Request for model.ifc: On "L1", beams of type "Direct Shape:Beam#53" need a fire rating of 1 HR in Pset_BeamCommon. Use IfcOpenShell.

First a look at what the model holds.

```python
import ifcopenshell
import ifcopenshell.util.element

model = ifcopenshell.open("model.ifc")
print(model.schema)
storey = next(s for s in model.by_type("IfcBuildingStorey") if s.Name == "L1")
beams = [e for e in ifcopenshell.util.element.get_decomposition(storey) if e.is_a("IfcBeam")]
seen = {}
for e in beams:
    element_type = ifcopenshell.util.element.get_type(e)
    key = (element_type.Name if element_type != e and element_type else None, ifcopenshell.util.element.get_pset(e, "Pset_BeamCommon", "FireRating"))
    seen[key] = seen.get(key, 0) + 1
for (name, value), count in sorted(seen.items(), key=str):
    print(count, "x", name, "|", value)
```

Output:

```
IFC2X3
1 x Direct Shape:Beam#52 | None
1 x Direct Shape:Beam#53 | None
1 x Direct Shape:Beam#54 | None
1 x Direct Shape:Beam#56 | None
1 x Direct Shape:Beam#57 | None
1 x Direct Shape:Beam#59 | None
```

```python
import ifcopenshell
import ifcopenshell.api.pset
import ifcopenshell.util.element

model = ifcopenshell.open("model.ifc")

storey = next(s for s in model.by_type("IfcBuildingStorey") if s.Name == "L1")
beams = [e for e in ifcopenshell.util.element.get_decomposition(storey) if e.is_a("IfcBeam")]

count = 0
for e in beams:
    element_type = ifcopenshell.util.element.get_type(e)
    if element_type in (None, e) or element_type.Name != "Direct Shape:Beam#53":
        continue
    # add_pset returns the element's existing set when there is one.
    pset = ifcopenshell.api.pset.add_pset(model, product=e, name="Pset_BeamCommon")
    ifcopenshell.api.pset.edit_pset(model, pset=pset, properties={"FireRating": "1 HR"})
    count += 1

print(count, "beams updated")

model.write("model_v2.ifc")
```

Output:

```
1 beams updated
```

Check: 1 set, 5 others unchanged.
